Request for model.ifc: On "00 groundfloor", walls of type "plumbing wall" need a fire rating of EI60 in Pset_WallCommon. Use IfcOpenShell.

First a look at what the model holds.

```python
import ifcopenshell
import ifcopenshell.util.element

model = ifcopenshell.open("model.ifc")
print(model.schema)
storey = next(s for s in model.by_type("IfcBuildingStorey") if s.Name == "00 groundfloor")
walls = [e for e in ifcopenshell.util.element.get_decomposition(storey) if e.is_a("IfcWall")]
seen = {}
for e in walls:
    element_type = ifcopenshell.util.element.get_type(e)
    key = (element_type.Name if element_type != e and element_type else None, ifcopenshell.util.element.get_pset(e, "Pset_WallCommon", "FireRating"))
    seen[key] = seen.get(key, 0) + 1
for (name, value), count in sorted(seen.items(), key=str):
    print(count, "x", name, "|", value)
```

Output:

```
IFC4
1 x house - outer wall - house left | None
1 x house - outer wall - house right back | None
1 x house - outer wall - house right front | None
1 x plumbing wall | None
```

```python
import ifcopenshell
import ifcopenshell.api.pset
import ifcopenshell.util.element

model = ifcopenshell.open("model.ifc")

storey = next(s for s in model.by_type("IfcBuildingStorey") if s.Name == "00 groundfloor")
walls = [e for e in ifcopenshell.util.element.get_decomposition(storey) if e.is_a("IfcWall")]

count = 0
for e in walls:
    element_type = ifcopenshell.util.element.get_type(e)
    if element_type in (None, e) or element_type.Name != "plumbing wall":
        continue
    # add_pset returns the element's existing set when there is one.
    pset = ifcopenshell.api.pset.add_pset(model, product=e, name="Pset_WallCommon")
    ifcopenshell.api.pset.edit_pset(model, pset=pset, properties={"FireRating": "EI60"})
    count += 1

print(count, "walls updated")

model.write("model_rev.ifc")
```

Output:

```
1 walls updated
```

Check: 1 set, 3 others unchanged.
